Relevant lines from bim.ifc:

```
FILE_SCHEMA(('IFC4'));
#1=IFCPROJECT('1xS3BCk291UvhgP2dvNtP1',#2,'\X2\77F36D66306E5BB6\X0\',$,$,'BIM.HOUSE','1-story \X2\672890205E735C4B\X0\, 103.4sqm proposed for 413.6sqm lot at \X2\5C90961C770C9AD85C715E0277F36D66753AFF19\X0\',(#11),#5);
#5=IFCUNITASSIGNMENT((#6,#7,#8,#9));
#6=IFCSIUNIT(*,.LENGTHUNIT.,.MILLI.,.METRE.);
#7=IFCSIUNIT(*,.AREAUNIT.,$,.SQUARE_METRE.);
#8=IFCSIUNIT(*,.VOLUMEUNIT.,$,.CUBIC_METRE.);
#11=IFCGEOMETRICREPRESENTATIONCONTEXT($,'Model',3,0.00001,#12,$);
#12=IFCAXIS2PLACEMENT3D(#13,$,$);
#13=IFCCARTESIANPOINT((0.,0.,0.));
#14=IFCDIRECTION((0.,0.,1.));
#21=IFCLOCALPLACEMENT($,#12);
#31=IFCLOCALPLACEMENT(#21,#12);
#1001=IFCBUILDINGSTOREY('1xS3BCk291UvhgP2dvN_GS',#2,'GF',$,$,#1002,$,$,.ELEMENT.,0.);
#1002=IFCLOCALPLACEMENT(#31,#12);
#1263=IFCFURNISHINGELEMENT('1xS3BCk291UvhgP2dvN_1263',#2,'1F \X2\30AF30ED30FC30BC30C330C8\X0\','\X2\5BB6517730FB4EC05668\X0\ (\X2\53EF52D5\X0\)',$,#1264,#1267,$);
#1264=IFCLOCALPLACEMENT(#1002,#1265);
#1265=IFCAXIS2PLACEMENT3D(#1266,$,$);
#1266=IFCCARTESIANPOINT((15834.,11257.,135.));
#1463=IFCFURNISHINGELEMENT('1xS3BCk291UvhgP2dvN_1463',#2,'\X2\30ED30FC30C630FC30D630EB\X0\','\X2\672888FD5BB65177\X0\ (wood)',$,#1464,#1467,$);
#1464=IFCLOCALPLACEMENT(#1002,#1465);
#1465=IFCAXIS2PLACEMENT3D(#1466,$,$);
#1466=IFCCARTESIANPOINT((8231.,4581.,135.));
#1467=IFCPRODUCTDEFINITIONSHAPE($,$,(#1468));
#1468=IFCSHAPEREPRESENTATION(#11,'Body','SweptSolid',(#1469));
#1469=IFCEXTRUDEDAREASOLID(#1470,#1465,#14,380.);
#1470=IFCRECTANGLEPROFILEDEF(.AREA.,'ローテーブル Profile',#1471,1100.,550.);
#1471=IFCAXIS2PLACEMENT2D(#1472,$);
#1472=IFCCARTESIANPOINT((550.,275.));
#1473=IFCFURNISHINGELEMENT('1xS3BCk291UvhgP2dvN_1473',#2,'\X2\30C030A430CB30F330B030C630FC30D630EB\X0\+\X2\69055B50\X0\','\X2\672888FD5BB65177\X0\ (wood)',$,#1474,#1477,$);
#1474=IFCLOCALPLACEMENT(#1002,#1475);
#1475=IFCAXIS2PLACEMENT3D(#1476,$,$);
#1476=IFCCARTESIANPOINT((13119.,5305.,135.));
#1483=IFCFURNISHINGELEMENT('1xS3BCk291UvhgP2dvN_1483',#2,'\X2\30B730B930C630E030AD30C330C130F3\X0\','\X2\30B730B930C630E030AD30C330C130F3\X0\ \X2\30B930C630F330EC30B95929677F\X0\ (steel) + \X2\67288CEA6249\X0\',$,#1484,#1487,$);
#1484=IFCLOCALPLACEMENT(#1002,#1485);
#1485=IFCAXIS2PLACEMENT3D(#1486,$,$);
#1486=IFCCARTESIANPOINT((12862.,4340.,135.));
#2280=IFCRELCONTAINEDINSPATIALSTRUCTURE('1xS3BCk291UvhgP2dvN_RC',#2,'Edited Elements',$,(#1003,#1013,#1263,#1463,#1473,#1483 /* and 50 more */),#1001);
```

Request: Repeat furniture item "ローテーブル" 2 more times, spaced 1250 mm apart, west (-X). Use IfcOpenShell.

```python
import numpy as np
import ifcopenshell
import ifcopenshell.api.geometry
import ifcopenshell.api.root
import ifcopenshell.util.element
import ifcopenshell.util.placement
import ifcopenshell.util.unit

model = ifcopenshell.open("bim.ifc")
unit_scale = ifcopenshell.util.unit.calculate_unit_scale(model)


def reuse_history(source, copy):
    """copy_class also copies each property set's owner history, people and application; keep the originals."""
    for rel in copy.IsDefinedBy:
        if rel.is_a("IfcRelDefinesByProperties") and (history := rel.RelatingPropertyDefinition.OwnerHistory):
            rel.RelatingPropertyDefinition.OwnerHistory = source.OwnerHistory
            ifcopenshell.util.element.remove_deep2(model, history)


source = model.by_guid("1xS3BCk291UvhgP2dvN_1463")
base = ifcopenshell.util.placement.get_local_placement(source.ObjectPlacement)
step = np.array([-1.0, 0.0, 0.0]) * 1.25 / unit_scale

for i in range(1, 3):
    copy = ifcopenshell.api.root.copy_class(model, product=source)
    copy.Representation = ifcopenshell.util.element.copy_deep(
        model, source.Representation, exclude=["IfcGeometricRepresentationContext", "IfcRepresentationMap"]
    )
    reuse_history(source, copy)
    matrix = base.copy()
    matrix[:3, 3] += i * step
    print("added at", matrix[:3, 3].round(3) + 0.0)
    ifcopenshell.api.geometry.edit_object_placement(model, product=copy, matrix=matrix, is_si=False)

model.write("bim-out.ifc")
```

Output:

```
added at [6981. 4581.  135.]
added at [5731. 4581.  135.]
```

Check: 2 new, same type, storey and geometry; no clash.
